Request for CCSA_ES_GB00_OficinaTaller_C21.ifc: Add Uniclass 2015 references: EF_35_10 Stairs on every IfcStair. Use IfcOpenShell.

First a look at what the model holds.

```python
import ifcopenshell

model = ifcopenshell.open("CCSA_ES_GB00_OficinaTaller_C21.ifc")
print(model.schema)
print("classifications:", [c.Name for c in model.by_type("IfcClassification")])
for ifc_class in ("IfcDoor", "IfcRoof", "IfcStair", "IfcWall", "IfcWindow"):
    print(ifc_class, len(model.by_type(ifc_class)))
```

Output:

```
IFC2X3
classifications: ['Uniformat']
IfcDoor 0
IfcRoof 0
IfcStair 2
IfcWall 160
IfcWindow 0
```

```python
import ifcopenshell
import ifcopenshell.api.classification

model = ifcopenshell.open("CCSA_ES_GB00_OficinaTaller_C21.ifc")

# IFC2X3 requires Source and Edition and has no link from the project to the system.
system = model.create_entity("IfcClassification", Source="NBS", Edition="2015", Name="Uniclass 2015")

codes = {
    "IfcStair": ("EF_35_10", "Stairs"),
}
for ifc_class, (code, name) in codes.items():
    products = model.by_type(ifc_class)
    ifcopenshell.api.classification.add_reference(
        model, products=products, classification=system, identification=code, name=name
    )
    print(code, len(products))

model.write("CCSA_ES_GB00_OficinaTaller_C21_v2.ifc")
```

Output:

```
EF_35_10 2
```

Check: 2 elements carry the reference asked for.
